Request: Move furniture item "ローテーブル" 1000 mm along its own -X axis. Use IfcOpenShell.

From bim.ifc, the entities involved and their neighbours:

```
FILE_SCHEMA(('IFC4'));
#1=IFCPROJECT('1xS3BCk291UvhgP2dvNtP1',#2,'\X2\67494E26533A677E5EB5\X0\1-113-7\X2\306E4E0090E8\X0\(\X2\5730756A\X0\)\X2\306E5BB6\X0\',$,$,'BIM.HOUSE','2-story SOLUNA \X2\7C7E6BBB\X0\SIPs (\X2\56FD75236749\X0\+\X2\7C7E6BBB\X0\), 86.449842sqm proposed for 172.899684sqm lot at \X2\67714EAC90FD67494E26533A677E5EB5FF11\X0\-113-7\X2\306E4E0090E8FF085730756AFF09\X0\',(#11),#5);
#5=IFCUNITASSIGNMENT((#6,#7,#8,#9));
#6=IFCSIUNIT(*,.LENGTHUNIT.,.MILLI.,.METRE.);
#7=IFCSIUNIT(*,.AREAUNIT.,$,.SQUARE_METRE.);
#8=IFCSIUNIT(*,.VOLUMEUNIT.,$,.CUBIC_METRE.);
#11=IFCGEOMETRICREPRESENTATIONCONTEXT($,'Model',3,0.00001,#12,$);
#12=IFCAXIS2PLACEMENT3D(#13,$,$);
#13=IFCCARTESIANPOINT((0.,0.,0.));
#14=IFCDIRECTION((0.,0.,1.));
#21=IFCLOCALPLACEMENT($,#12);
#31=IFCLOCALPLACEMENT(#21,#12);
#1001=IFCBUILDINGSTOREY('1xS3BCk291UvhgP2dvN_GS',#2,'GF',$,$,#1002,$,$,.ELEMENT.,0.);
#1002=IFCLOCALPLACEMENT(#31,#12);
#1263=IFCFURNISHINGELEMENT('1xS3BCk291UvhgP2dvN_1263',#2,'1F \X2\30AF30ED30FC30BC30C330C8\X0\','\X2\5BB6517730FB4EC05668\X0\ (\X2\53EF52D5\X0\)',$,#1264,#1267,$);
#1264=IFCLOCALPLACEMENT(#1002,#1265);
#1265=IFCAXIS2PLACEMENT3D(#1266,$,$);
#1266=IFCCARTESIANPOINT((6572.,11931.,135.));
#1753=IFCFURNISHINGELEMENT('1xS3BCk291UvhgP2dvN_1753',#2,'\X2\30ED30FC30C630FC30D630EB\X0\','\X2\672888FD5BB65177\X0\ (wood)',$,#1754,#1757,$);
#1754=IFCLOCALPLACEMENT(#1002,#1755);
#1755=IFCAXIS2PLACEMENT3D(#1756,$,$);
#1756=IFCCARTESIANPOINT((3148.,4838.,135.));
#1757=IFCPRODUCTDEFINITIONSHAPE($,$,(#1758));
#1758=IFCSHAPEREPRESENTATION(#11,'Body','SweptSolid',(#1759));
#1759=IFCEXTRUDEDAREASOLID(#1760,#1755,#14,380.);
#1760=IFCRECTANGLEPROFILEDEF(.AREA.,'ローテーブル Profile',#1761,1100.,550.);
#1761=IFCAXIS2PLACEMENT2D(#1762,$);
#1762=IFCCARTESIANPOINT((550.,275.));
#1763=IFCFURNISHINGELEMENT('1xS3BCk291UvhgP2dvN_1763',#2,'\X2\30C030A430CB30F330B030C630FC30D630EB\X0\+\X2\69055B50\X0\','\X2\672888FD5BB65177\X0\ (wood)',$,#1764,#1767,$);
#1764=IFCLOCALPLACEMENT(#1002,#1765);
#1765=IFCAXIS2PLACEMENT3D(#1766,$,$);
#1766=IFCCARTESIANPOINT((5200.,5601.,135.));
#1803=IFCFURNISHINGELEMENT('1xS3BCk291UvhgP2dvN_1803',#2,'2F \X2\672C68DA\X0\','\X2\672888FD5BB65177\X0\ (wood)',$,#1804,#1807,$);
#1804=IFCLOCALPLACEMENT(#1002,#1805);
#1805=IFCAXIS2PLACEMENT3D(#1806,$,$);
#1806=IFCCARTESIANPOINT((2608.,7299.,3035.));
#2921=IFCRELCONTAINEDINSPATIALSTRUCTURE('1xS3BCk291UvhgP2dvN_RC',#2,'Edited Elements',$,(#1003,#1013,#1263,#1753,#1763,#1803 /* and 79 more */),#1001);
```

```python
import ifcopenshell
import ifcopenshell.api.geometry
import ifcopenshell.util.placement

model = ifcopenshell.open("bim.ifc")

item = model.by_id(1753)
matrix = ifcopenshell.util.placement.get_local_placement(item.ObjectPlacement)
matrix[:3, 3] -= matrix[:3, 0] * 1000.0
ifcopenshell.api.geometry.edit_object_placement(model, product=item, matrix=matrix, is_si=False)

print(ifcopenshell.util.placement.get_local_placement(item.ObjectPlacement).round(3) + 0.0)

model.write("bim_v2.ifc")
```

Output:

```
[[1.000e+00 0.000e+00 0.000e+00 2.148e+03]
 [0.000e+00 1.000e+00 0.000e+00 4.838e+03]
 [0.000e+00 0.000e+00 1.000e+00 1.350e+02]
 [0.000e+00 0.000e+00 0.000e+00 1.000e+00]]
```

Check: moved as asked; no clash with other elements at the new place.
